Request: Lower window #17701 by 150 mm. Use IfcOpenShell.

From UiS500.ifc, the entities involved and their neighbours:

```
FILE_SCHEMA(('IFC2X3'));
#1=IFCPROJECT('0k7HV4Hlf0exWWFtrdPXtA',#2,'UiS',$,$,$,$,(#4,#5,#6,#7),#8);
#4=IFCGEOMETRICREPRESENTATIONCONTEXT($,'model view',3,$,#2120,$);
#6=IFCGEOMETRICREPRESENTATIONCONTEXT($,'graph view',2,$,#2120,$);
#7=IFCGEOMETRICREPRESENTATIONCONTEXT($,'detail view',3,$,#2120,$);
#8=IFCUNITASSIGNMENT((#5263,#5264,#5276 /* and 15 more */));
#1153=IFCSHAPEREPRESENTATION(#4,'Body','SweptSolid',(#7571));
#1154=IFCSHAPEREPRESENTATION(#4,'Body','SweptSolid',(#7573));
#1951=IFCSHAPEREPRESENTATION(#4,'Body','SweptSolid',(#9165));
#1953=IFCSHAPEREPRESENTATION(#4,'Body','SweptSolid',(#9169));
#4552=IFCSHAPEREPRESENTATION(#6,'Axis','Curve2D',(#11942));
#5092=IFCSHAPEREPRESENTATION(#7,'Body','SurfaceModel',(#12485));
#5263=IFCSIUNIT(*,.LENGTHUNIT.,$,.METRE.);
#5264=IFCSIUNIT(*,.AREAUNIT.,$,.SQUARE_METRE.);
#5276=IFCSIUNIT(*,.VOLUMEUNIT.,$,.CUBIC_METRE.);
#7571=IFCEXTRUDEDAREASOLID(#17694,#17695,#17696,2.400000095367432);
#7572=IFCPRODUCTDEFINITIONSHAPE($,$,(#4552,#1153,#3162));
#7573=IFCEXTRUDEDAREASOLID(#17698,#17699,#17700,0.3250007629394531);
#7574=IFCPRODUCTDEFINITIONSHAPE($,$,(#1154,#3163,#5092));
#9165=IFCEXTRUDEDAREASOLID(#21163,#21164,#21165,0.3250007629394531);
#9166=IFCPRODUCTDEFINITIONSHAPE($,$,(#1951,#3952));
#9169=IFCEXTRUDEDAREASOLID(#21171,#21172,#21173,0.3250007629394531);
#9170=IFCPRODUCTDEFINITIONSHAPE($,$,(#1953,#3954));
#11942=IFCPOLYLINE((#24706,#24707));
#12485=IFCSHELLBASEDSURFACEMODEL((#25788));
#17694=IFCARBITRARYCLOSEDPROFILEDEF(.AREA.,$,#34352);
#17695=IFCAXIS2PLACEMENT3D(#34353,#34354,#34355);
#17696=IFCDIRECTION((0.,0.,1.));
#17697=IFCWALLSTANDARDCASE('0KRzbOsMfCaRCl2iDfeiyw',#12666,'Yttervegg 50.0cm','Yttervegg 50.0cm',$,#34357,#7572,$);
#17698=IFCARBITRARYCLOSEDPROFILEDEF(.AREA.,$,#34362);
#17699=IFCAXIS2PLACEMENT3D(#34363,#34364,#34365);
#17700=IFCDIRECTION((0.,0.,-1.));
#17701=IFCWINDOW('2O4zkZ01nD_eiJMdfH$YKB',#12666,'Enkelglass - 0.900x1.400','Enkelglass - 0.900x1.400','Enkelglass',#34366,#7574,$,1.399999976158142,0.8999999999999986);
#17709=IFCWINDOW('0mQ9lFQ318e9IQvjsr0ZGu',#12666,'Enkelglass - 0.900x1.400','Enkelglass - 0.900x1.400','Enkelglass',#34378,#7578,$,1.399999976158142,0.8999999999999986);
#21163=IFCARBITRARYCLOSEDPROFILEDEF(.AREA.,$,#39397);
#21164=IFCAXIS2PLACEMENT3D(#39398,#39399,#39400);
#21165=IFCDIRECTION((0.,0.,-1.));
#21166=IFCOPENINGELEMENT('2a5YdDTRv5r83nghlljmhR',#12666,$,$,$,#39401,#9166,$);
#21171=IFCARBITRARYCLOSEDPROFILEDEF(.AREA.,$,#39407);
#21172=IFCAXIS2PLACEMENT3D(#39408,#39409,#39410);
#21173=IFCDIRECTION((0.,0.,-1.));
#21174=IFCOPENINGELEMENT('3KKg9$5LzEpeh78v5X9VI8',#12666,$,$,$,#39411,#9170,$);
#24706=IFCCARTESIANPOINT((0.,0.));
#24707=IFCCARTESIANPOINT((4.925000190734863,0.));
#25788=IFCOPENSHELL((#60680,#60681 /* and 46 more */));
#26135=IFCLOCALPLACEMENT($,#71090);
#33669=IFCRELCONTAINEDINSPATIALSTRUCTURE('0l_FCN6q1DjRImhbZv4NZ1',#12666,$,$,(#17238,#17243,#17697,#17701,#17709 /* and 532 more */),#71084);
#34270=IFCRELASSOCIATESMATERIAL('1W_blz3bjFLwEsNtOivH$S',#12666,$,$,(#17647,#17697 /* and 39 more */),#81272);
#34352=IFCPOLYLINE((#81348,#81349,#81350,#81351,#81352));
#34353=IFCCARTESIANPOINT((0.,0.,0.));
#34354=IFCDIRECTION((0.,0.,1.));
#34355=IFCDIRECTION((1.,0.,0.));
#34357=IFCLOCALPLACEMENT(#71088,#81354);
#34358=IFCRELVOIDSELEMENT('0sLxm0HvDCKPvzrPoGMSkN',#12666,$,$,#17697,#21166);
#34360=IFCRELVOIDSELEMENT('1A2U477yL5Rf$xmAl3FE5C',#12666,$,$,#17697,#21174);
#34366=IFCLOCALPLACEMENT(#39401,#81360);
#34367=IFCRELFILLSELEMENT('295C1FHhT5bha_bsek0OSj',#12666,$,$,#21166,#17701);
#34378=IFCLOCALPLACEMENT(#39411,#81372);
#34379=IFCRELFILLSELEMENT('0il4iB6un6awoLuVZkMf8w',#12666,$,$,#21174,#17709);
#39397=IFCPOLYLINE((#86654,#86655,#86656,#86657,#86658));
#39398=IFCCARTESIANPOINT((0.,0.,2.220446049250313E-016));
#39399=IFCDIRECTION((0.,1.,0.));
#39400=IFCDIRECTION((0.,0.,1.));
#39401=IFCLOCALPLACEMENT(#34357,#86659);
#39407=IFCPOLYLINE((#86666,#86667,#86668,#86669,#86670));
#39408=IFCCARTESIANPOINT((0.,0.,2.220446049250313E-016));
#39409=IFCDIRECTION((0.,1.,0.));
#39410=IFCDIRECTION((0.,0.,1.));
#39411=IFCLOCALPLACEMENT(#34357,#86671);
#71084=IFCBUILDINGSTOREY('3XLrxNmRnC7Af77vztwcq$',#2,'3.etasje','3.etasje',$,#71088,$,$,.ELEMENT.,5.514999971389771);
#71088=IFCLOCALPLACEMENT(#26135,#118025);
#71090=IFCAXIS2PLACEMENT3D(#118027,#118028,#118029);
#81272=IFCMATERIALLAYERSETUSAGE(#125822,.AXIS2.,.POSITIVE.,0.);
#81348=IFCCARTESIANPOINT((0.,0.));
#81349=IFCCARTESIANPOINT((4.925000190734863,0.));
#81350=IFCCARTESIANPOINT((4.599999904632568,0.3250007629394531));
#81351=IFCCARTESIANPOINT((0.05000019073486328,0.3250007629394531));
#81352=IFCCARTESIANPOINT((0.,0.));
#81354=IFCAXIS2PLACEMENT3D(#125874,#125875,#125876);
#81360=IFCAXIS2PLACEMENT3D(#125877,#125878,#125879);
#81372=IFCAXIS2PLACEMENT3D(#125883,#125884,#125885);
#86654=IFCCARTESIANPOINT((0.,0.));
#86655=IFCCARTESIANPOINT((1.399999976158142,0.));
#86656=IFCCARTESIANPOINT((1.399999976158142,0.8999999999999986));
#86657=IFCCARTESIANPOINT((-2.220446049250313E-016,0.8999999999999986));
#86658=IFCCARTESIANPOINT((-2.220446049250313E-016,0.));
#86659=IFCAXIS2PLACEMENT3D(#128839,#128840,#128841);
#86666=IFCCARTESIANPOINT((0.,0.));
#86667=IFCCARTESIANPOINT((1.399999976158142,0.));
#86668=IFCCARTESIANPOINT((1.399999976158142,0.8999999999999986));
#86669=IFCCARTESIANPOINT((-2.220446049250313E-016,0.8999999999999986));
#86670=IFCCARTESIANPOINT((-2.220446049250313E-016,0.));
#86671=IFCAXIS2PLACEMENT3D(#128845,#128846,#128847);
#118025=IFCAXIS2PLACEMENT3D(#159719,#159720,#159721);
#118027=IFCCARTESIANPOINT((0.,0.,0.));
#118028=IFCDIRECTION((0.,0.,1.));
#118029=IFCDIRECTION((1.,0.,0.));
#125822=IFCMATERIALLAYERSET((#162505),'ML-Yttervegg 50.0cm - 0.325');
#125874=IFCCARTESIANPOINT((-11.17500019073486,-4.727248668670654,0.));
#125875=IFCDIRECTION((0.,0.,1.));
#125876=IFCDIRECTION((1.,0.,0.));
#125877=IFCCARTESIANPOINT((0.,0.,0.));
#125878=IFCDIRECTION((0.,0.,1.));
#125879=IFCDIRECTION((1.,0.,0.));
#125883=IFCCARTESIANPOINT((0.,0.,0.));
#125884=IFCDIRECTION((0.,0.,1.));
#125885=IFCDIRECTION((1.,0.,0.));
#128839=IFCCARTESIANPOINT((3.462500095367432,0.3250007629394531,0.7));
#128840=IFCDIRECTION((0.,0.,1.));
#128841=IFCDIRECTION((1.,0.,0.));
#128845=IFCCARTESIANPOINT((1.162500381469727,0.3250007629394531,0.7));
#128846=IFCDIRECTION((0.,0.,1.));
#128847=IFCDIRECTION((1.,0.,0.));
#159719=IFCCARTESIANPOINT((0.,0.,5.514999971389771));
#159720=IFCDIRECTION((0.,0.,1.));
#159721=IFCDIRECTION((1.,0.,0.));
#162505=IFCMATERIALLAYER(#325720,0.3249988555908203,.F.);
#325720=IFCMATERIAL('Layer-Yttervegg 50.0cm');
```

```python
import numpy as np
import ifcopenshell
import ifcopenshell.api.geometry
import ifcopenshell.util.placement
import ifcopenshell.util.unit

model = ifcopenshell.open("UiS500.ifc")
unit_scale = ifcopenshell.util.unit.calculate_unit_scale(model)

window = model.by_guid("2O4zkZ01nD_eiJMdfH$YKB")
opening = window.FillsVoids[0].RelatingOpeningElement
dz = -0.15

shift = np.array([0.0, 0.0, dz])
# The window is placed relative to its opening, so it follows when the opening moves.
matrix = ifcopenshell.util.placement.get_local_placement(opening.ObjectPlacement)
matrix[:3, 3] += shift
ifcopenshell.api.geometry.edit_object_placement(
    model, product=opening, matrix=matrix, is_si=False, should_transform_children=True
)

print(f"moved by {dz * unit_scale:+.3f} m")

model.write("UiS500_v2.ifc")
```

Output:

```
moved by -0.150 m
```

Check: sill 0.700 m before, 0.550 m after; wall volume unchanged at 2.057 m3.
